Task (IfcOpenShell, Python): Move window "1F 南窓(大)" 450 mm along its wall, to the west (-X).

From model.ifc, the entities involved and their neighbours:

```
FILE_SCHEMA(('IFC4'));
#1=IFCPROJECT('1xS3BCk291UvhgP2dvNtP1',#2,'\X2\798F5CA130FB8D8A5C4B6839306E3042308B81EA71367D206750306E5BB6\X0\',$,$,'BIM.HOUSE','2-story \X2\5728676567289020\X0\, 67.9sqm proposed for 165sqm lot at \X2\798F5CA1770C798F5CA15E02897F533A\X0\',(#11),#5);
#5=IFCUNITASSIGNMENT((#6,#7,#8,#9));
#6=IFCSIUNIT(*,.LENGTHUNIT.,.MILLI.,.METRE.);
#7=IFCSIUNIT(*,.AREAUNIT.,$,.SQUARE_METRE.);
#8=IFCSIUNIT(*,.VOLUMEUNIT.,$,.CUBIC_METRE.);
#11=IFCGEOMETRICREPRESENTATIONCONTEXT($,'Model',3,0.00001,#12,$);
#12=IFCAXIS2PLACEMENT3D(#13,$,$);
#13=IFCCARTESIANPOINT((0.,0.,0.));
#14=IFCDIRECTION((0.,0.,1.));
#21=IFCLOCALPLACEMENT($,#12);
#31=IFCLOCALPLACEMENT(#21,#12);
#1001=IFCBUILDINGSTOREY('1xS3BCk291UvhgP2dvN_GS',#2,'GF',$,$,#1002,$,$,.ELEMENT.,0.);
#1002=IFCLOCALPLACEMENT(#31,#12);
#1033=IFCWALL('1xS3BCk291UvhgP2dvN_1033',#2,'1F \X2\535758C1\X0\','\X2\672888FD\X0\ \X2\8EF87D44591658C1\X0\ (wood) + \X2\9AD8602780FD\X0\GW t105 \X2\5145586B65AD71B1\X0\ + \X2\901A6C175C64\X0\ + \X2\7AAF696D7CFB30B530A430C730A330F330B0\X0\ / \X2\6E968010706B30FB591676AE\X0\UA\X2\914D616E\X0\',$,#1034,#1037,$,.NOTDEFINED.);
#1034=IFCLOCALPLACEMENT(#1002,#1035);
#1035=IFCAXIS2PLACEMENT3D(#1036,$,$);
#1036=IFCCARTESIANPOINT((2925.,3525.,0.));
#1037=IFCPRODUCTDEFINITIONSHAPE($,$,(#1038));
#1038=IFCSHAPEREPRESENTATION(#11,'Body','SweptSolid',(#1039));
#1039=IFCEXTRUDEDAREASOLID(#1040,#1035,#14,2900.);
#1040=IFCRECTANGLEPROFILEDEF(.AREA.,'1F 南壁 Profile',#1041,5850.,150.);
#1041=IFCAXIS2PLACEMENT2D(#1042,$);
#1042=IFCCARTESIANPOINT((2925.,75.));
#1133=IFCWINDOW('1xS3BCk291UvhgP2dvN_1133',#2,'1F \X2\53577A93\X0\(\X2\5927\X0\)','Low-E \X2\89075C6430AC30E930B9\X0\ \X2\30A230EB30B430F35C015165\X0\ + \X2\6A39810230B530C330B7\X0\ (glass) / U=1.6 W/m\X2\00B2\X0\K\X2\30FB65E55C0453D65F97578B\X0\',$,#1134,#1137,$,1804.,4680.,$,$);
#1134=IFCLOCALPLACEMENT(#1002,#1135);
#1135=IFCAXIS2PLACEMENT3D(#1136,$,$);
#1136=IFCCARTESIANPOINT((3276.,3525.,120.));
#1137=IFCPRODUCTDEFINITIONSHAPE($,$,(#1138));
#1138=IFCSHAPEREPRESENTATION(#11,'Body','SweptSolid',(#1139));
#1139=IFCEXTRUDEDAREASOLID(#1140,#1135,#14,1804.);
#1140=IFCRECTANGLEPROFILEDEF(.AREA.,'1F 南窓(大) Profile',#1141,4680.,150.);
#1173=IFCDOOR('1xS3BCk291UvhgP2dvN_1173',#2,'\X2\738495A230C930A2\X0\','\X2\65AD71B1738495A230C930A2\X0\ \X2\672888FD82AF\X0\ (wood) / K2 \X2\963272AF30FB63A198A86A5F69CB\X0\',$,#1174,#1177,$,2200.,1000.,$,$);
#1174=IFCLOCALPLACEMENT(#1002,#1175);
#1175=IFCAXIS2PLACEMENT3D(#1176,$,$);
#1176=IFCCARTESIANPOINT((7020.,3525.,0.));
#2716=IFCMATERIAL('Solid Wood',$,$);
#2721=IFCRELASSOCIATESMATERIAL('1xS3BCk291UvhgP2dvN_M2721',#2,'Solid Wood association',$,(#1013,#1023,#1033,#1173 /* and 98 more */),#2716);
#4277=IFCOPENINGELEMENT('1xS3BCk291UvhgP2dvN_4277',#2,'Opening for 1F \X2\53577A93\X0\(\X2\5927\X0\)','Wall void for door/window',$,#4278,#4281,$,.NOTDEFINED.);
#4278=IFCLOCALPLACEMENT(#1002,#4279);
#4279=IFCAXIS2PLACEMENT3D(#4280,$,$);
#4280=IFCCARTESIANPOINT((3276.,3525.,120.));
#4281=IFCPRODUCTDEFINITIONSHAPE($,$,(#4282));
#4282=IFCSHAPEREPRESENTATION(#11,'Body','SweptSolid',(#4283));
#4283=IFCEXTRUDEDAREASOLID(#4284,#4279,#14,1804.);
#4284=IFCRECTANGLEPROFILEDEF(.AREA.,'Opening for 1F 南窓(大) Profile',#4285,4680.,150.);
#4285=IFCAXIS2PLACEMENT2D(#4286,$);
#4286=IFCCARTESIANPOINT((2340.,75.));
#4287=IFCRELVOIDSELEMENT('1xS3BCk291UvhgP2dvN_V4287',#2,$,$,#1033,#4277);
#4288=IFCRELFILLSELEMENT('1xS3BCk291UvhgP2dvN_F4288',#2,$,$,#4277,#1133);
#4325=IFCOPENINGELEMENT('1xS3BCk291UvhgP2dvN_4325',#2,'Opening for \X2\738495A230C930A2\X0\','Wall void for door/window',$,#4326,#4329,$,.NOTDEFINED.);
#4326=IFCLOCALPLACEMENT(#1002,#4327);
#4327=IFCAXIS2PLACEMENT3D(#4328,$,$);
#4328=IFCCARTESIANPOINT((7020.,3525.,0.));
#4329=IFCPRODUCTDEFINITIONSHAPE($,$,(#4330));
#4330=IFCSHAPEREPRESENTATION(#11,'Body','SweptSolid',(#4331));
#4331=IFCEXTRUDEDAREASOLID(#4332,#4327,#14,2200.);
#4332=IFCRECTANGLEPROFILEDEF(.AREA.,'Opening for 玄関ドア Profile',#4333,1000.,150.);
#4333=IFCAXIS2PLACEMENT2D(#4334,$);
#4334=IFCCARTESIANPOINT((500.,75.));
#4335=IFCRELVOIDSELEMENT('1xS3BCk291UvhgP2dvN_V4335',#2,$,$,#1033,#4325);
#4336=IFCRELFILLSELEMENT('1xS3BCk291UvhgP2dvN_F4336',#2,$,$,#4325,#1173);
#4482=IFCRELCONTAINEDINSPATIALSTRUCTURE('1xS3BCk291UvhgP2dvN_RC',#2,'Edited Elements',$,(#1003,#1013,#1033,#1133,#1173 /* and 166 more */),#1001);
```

```python
import ifcopenshell
import ifcopenshell.api.geometry
import ifcopenshell.util.placement

model = ifcopenshell.open("model.ifc")

window = model.by_guid("1xS3BCk291UvhgP2dvN_1133")
opening = window.FillsVoids[0].RelatingOpeningElement
wall = opening.VoidsElements[0].RelatingBuildingElement

wall_matrix = ifcopenshell.util.placement.get_local_placement(wall.ObjectPlacement)
shift = wall_matrix[:3, 0] * -450.0
before = ifcopenshell.util.placement.get_local_placement(window.ObjectPlacement)[:3, 3].copy()

# The window is not placed relative to its opening, so move both.
for product in (opening, window):
    matrix = ifcopenshell.util.placement.get_local_placement(product.ObjectPlacement)
    matrix[:3, 3] += shift
    ifcopenshell.api.geometry.edit_object_placement(model, product=product, matrix=matrix, is_si=False)

after = ifcopenshell.util.placement.get_local_placement(window.ObjectPlacement)[:3, 3]
print("window moved by", (after - before).round(3) + 0.0)

model.write("model_edited.ifc")
```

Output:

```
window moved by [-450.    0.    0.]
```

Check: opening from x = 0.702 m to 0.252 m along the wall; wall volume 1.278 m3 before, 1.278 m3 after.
